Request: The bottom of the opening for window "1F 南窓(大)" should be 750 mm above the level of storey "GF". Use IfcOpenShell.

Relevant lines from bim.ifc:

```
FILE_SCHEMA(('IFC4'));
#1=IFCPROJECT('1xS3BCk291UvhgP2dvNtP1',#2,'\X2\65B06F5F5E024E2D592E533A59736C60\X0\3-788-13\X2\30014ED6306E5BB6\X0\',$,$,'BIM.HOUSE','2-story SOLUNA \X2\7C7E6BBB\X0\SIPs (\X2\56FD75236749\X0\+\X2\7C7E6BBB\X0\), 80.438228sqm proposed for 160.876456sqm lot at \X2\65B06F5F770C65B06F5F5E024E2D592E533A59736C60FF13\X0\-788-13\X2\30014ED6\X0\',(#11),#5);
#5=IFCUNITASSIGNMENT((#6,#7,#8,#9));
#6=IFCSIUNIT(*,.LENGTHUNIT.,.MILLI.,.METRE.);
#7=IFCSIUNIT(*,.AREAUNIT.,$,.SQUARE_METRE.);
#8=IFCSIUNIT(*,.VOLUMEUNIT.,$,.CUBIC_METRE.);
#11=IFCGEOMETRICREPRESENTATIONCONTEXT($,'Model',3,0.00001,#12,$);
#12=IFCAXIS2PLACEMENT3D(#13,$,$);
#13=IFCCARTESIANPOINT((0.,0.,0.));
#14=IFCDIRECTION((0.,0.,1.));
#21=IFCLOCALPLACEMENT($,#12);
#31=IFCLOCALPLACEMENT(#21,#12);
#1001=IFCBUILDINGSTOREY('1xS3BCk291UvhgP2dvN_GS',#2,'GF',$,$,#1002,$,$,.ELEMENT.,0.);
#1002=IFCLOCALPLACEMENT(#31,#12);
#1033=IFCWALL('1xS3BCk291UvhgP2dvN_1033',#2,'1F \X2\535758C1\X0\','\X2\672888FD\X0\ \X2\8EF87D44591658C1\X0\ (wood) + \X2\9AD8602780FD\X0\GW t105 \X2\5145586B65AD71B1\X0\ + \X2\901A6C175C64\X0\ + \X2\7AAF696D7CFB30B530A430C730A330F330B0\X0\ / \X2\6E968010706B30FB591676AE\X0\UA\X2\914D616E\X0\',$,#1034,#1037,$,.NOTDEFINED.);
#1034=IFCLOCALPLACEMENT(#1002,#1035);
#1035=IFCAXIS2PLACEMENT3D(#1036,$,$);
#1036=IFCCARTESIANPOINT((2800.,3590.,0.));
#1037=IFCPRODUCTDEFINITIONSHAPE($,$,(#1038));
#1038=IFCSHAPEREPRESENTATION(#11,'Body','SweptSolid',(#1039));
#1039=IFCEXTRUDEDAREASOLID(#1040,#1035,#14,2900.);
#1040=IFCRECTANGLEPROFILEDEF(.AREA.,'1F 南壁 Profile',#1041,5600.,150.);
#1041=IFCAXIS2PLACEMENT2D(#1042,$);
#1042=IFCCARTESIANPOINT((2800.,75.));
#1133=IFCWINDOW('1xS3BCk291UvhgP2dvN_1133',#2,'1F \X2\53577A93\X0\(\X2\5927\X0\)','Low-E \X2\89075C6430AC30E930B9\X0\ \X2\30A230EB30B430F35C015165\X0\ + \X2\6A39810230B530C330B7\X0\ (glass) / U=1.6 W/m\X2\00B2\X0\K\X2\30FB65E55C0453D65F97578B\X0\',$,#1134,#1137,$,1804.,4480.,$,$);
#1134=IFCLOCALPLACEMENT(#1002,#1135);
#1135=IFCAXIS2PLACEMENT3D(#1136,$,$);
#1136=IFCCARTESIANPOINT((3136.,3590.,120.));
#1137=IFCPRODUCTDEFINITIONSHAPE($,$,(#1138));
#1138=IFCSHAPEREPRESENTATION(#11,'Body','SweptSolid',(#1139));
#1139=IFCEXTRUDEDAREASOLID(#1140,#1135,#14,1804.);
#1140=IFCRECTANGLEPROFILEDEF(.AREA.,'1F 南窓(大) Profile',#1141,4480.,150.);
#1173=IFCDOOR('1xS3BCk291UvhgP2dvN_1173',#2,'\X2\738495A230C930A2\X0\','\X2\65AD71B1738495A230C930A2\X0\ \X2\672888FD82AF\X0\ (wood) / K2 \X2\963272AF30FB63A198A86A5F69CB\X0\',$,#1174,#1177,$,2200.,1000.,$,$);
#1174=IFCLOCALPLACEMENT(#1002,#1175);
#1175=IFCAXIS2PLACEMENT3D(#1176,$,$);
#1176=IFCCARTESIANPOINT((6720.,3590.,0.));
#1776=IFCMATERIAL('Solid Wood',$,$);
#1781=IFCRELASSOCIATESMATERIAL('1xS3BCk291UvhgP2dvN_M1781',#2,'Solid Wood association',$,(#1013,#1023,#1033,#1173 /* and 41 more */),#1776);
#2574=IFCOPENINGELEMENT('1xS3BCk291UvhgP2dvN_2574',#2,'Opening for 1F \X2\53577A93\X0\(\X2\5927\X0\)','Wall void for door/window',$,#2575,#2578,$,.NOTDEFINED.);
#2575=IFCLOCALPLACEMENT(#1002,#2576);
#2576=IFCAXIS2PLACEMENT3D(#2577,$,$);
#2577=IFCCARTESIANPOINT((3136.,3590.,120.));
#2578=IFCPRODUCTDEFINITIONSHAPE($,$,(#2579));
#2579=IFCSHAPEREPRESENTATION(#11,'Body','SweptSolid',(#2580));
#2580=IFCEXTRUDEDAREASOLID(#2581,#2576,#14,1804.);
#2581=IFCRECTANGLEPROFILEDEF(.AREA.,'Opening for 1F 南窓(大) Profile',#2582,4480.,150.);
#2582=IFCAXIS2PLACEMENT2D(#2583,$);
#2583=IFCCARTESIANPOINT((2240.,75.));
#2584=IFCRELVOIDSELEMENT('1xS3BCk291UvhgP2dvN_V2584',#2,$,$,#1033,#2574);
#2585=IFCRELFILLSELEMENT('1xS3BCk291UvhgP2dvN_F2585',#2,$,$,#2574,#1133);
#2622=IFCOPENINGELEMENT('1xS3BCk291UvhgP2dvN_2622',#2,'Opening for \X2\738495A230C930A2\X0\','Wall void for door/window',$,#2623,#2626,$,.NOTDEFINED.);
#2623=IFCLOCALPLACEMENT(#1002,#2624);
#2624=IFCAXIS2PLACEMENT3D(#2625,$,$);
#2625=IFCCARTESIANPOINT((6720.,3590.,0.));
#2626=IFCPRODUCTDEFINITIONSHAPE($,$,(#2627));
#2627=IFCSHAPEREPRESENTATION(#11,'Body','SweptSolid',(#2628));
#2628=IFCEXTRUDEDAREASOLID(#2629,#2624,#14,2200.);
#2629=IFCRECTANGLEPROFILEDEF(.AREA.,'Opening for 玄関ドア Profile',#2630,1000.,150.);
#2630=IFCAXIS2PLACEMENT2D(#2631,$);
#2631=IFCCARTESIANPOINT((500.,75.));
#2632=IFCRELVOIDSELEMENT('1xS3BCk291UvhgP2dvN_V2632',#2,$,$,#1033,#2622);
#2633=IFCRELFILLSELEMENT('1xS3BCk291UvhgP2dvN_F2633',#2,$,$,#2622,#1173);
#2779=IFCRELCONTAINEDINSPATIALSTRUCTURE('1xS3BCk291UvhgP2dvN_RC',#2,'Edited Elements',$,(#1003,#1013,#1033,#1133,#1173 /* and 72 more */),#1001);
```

```python
import numpy as np
import ifcopenshell
import ifcopenshell.api.geometry
import ifcopenshell.geom
import ifcopenshell.util.element
import ifcopenshell.util.placement
import ifcopenshell.util.shape
import ifcopenshell.util.unit

model = ifcopenshell.open("bim.ifc")
unit_scale = ifcopenshell.util.unit.calculate_unit_scale(model)

window = model.by_guid("1xS3BCk291UvhgP2dvN_1133")
opening = window.FillsVoids[0].RelatingOpeningElement
storey = ifcopenshell.util.element.get_container(window, ifc_class="IfcBuildingStorey")
level = ifcopenshell.util.placement.get_local_placement(storey.ObjectPlacement)[2, 3]

# The opening's origin need not be at the sill, so measure its lowest point.
shape = ifcopenshell.geom.create_shape(ifcopenshell.geom.settings(), opening)
bottom = ifcopenshell.util.shape.get_shape_bottom_elevation(shape, shape.geometry) / unit_scale
dz = level + 750.0 - bottom

shift = np.array([0.0, 0.0, dz])
# The window is not placed relative to its opening, so move both.
for product in (opening, window):
    matrix = ifcopenshell.util.placement.get_local_placement(product.ObjectPlacement)
    matrix[:3, 3] += shift
    ifcopenshell.api.geometry.edit_object_placement(model, product=product, matrix=matrix, is_si=False)

print(f"moved by {dz * unit_scale:+.3f} m")

model.write("bim_rev.ifc")
```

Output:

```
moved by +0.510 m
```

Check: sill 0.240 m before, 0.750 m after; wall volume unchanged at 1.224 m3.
